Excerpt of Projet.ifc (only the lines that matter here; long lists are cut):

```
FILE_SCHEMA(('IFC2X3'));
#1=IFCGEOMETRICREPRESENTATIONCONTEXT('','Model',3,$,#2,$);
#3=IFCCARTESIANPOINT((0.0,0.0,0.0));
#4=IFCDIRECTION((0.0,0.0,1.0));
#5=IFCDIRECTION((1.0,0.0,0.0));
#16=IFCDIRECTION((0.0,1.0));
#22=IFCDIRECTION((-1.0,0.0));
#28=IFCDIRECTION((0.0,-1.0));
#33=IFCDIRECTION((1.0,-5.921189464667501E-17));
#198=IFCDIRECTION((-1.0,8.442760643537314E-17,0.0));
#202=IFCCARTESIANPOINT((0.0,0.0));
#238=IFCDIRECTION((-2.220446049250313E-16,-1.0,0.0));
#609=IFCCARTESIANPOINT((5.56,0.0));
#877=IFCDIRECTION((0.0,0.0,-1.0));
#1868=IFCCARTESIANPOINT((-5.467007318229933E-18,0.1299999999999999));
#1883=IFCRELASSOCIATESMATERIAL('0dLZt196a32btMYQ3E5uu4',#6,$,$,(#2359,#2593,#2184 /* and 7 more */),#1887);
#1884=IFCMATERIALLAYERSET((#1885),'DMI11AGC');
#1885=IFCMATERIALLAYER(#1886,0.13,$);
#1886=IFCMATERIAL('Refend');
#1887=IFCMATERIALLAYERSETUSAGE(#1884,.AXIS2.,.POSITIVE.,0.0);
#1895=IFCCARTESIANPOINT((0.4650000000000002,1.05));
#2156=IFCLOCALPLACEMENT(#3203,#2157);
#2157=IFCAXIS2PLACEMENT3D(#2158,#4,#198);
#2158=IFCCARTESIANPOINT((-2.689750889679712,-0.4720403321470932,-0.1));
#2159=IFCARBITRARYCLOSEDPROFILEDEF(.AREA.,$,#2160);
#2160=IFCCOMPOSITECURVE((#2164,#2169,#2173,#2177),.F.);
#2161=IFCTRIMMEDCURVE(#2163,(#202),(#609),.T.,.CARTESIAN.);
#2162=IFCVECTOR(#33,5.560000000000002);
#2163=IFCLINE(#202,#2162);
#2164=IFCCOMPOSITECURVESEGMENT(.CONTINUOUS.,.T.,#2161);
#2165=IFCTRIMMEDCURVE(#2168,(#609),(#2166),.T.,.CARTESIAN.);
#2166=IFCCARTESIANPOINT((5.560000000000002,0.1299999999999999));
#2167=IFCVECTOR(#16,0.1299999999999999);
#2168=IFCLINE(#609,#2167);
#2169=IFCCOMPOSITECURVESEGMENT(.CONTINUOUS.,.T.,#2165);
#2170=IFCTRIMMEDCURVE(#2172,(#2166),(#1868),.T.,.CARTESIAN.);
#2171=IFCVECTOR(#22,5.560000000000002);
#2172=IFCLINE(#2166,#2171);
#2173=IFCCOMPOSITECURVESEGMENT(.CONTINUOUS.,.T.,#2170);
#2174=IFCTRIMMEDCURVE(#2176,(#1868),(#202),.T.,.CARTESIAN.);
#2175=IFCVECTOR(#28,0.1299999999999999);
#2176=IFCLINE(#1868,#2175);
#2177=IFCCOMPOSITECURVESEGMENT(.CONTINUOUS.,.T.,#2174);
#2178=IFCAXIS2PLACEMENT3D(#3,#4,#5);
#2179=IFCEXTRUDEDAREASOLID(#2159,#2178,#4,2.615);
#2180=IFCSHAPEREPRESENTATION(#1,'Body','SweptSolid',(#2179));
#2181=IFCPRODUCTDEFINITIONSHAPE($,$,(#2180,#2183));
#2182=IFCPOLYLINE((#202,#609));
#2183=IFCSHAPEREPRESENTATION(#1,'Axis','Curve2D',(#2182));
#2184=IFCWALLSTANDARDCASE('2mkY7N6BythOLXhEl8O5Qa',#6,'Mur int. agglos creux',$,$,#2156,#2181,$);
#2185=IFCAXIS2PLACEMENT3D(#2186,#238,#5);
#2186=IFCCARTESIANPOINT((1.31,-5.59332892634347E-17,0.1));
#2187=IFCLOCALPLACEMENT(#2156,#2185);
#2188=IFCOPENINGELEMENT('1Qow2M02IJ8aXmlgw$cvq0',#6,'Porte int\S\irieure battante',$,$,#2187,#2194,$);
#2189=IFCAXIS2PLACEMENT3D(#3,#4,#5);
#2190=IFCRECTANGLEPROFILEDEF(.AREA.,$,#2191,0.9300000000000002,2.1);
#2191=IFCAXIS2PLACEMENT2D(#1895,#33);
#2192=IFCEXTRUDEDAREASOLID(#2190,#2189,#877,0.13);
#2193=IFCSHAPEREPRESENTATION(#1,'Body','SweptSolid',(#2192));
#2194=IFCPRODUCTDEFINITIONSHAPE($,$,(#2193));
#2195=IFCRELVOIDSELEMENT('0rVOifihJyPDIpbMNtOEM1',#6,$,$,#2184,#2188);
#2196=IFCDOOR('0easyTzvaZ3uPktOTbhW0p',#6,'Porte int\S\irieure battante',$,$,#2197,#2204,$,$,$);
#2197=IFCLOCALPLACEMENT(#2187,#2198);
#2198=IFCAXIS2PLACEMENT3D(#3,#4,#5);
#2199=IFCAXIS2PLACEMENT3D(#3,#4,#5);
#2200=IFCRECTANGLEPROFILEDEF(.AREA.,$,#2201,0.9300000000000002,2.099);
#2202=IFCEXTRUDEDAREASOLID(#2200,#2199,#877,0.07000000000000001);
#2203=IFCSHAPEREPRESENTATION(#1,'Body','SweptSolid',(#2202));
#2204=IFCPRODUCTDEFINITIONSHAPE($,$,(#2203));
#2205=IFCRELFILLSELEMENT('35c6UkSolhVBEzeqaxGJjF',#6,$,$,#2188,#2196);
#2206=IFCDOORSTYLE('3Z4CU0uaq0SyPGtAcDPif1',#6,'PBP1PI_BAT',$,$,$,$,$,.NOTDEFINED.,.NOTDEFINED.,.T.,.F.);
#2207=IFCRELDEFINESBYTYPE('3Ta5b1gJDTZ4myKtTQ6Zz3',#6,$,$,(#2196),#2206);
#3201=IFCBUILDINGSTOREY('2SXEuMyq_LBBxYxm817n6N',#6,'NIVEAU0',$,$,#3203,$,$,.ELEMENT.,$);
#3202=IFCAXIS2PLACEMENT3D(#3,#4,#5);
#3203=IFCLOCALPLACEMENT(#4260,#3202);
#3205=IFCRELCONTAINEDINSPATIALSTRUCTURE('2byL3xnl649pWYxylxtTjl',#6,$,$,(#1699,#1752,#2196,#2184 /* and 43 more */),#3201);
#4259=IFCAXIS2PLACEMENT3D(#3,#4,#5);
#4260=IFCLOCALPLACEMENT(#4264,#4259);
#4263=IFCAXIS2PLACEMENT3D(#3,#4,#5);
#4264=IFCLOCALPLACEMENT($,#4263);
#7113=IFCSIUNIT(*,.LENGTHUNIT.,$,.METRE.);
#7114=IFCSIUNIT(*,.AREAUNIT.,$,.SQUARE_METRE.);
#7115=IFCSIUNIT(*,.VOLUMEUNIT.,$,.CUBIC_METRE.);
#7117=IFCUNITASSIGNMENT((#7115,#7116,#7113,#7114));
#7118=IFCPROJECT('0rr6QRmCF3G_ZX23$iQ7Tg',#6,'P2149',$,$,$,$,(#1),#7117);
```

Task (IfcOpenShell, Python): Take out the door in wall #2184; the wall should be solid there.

```python
import ifcopenshell
import ifcopenshell.api.feature
import ifcopenshell.api.root
import ifcopenshell.geom
import ifcopenshell.util.shape

model = ifcopenshell.open("Projet.ifc")
settings = ifcopenshell.geom.settings()


def volume(element):
    """Net volume in cubic metres, openings subtracted."""
    shape = ifcopenshell.geom.create_shape(settings, element)
    return ifcopenshell.util.shape.get_volume(shape.geometry)


door = model.by_id(2196)
opening = door.FillsVoids[0].RelatingOpeningElement
wall = opening.VoidsElements[0].RelatingBuildingElement
before = volume(wall)

ifcopenshell.api.root.remove_product(model, product=door)
ifcopenshell.api.feature.remove_feature(model, feature=opening)

after = volume(wall)

print(f"wall volume {before:.3f} -> {after:.3f} m3")

model.write("Projet-out.ifc")
```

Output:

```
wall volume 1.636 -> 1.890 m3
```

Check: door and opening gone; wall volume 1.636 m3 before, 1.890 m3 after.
